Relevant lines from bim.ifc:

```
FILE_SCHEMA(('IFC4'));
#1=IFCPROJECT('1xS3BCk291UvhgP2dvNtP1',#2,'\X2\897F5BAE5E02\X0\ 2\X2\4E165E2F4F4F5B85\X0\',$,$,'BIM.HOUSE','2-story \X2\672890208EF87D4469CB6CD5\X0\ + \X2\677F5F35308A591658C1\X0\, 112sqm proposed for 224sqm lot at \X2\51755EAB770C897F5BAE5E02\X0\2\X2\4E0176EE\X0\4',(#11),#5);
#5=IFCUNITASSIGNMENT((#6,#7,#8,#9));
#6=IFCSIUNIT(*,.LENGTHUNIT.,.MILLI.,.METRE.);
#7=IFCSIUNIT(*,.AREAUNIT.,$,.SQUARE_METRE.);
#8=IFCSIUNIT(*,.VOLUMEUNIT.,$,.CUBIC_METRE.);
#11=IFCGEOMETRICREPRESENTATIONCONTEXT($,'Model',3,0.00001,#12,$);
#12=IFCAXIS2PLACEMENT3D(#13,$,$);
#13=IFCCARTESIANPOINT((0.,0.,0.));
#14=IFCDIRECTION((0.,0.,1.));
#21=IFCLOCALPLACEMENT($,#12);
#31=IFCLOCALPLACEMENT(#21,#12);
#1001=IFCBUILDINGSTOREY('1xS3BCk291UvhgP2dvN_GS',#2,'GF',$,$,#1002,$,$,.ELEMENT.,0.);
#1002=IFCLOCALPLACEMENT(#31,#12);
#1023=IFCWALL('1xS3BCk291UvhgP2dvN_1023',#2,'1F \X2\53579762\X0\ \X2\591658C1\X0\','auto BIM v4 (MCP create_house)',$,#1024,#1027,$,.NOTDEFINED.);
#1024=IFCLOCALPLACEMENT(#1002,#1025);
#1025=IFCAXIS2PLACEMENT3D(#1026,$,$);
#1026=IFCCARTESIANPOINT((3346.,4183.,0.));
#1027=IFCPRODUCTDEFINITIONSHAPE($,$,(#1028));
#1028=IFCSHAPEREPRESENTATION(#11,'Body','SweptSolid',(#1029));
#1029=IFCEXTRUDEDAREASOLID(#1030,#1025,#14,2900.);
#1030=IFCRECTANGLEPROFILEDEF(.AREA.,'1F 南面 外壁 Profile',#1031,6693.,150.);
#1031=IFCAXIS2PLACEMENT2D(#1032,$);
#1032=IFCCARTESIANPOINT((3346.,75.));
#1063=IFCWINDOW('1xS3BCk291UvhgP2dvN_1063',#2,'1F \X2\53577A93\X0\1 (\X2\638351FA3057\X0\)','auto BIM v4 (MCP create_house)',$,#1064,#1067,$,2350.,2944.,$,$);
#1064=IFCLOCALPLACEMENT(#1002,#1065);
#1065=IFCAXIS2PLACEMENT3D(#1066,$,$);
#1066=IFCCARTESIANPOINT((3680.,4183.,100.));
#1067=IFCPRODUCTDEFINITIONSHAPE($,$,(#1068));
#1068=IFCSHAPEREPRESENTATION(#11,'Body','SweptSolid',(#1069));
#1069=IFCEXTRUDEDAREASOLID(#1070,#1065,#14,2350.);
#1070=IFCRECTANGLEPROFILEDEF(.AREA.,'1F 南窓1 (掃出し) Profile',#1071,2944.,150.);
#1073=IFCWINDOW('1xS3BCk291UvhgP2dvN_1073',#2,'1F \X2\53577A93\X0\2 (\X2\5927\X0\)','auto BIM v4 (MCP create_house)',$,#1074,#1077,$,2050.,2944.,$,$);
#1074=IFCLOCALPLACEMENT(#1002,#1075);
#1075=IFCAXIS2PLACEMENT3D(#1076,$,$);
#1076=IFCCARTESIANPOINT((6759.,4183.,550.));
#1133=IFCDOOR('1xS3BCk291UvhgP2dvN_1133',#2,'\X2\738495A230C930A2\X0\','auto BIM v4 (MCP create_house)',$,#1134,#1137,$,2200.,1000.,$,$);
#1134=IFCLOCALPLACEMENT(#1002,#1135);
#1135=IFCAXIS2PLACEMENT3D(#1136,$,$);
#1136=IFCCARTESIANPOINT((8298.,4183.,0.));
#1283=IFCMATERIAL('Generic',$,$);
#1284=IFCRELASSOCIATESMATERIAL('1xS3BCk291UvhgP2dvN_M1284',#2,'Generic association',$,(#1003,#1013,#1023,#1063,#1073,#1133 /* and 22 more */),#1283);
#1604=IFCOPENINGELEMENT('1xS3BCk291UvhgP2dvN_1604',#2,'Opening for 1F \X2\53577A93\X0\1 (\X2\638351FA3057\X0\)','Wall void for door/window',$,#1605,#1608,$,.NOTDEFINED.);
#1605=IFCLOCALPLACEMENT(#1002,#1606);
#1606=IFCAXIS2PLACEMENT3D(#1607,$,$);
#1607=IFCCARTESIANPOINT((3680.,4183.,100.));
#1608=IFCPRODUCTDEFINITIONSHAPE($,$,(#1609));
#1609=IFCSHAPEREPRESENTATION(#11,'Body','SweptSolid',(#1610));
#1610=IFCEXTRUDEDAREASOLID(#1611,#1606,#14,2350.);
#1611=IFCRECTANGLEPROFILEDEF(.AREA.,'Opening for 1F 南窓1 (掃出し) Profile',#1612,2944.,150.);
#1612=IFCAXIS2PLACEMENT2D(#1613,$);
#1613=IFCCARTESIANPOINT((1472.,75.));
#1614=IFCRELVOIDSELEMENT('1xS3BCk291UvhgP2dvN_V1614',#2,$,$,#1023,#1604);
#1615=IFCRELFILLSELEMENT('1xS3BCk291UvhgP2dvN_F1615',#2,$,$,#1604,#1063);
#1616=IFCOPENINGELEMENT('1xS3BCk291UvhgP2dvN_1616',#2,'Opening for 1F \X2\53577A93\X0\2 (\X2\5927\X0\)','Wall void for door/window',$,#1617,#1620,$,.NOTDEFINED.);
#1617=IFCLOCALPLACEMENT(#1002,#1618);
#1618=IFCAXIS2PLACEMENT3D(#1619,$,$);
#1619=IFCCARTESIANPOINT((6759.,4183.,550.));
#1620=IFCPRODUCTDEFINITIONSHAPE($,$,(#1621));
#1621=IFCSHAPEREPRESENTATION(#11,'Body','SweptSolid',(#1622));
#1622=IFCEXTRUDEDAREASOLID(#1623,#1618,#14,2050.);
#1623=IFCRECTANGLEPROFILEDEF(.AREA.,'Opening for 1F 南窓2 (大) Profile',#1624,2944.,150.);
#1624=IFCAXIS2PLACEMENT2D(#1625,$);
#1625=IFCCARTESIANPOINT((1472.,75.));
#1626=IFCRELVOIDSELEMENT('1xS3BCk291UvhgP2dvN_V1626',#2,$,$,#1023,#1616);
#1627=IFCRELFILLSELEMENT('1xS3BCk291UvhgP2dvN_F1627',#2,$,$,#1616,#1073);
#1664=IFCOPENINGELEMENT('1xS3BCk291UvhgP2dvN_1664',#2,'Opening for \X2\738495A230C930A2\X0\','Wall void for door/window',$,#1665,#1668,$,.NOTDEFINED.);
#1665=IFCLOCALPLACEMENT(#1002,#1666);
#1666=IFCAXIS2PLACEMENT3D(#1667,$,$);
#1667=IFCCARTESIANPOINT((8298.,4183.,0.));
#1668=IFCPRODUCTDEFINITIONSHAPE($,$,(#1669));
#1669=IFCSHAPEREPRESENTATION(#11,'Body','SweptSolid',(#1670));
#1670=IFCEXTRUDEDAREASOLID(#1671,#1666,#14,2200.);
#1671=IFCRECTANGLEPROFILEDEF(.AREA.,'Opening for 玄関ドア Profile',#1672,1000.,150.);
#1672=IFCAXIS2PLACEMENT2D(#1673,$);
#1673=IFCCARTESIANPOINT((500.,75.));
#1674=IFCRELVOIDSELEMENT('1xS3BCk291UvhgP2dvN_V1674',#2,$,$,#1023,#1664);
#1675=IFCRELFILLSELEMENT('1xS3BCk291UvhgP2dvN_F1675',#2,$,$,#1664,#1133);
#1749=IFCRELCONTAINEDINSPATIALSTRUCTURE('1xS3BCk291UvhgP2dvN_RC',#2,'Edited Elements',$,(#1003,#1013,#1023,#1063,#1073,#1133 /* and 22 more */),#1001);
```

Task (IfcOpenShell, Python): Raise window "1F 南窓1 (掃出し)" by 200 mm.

```python
import numpy as np
import ifcopenshell
import ifcopenshell.api.geometry
import ifcopenshell.util.placement
import ifcopenshell.util.unit

model = ifcopenshell.open("bim.ifc")
unit_scale = ifcopenshell.util.unit.calculate_unit_scale(model)

window = model.by_guid("1xS3BCk291UvhgP2dvN_1063")
opening = window.FillsVoids[0].RelatingOpeningElement
dz = 0.2 / unit_scale

shift = np.array([0.0, 0.0, dz])
# The window is not placed relative to its opening, so move both.
for product in (opening, window):
    matrix = ifcopenshell.util.placement.get_local_placement(product.ObjectPlacement)
    matrix[:3, 3] += shift
    ifcopenshell.api.geometry.edit_object_placement(model, product=product, matrix=matrix, is_si=False)

print(f"moved by {dz * unit_scale:+.3f} m")

model.write("bim_v2.ifc")
```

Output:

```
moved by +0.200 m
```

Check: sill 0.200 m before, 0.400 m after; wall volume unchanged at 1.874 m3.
